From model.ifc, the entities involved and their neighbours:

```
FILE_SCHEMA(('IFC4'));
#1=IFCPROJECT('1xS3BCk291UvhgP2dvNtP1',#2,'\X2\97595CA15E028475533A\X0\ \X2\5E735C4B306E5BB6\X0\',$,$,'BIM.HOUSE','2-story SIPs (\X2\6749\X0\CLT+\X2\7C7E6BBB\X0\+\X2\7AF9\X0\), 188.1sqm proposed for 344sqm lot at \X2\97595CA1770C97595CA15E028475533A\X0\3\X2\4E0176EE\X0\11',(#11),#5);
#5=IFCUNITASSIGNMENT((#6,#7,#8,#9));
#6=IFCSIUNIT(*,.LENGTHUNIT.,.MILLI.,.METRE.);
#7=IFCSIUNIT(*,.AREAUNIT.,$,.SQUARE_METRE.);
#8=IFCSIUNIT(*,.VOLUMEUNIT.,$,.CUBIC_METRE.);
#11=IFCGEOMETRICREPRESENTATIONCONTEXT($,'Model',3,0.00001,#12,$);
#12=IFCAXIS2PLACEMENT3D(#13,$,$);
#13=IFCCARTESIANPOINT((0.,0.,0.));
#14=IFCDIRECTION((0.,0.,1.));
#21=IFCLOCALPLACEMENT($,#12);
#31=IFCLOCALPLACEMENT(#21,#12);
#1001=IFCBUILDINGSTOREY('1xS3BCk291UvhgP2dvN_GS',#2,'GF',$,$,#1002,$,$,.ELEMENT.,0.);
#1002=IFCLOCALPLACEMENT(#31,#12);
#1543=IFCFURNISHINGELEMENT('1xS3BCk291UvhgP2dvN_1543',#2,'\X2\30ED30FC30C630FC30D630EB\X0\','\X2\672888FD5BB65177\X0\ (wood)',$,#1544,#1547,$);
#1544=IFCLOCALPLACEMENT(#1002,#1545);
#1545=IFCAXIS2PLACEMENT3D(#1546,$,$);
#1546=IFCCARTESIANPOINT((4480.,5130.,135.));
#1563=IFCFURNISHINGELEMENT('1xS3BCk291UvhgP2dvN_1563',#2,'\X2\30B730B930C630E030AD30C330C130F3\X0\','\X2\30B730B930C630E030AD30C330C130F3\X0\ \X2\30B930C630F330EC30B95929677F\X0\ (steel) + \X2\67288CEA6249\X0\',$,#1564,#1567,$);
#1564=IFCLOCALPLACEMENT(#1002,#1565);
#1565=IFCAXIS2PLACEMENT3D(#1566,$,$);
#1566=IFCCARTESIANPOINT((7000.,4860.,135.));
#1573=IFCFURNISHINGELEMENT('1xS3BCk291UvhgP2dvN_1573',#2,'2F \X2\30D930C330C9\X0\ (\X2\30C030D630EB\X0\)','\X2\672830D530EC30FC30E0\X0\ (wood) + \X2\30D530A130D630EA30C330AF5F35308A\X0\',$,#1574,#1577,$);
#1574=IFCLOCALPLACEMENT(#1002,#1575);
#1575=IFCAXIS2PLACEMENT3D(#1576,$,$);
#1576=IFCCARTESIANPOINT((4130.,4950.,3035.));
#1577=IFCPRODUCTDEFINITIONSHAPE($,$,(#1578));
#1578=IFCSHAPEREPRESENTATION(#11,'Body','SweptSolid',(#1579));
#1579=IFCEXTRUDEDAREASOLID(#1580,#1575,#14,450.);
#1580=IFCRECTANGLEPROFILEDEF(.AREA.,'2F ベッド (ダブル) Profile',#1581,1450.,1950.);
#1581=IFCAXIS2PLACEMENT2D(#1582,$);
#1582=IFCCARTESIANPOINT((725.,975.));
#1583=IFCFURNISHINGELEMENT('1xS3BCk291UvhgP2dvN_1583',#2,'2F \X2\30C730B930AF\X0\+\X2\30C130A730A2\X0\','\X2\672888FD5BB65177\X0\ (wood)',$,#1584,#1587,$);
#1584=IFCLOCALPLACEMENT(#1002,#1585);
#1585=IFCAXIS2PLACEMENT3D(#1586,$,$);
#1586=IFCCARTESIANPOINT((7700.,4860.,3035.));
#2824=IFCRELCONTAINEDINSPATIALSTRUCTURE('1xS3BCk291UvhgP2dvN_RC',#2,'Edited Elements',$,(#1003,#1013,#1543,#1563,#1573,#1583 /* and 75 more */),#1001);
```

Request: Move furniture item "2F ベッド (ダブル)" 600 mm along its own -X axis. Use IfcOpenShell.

```python
import ifcopenshell
import ifcopenshell.api.geometry
import ifcopenshell.util.placement
import ifcopenshell.util.unit

model = ifcopenshell.open("model.ifc")
unit_scale = ifcopenshell.util.unit.calculate_unit_scale(model)

item = model.by_guid("1xS3BCk291UvhgP2dvN_1573")
matrix = ifcopenshell.util.placement.get_local_placement(item.ObjectPlacement)
matrix[:3, 3] -= matrix[:3, 0] * 0.6 / unit_scale
ifcopenshell.api.geometry.edit_object_placement(model, product=item, matrix=matrix, is_si=False)

print(ifcopenshell.util.placement.get_local_placement(item.ObjectPlacement).round(3) + 0.0)

model.write("model_edited.ifc")
```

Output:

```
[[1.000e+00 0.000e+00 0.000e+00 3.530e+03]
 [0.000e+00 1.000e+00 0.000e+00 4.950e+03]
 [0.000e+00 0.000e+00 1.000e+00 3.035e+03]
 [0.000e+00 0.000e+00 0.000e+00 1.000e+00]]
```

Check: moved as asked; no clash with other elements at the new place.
